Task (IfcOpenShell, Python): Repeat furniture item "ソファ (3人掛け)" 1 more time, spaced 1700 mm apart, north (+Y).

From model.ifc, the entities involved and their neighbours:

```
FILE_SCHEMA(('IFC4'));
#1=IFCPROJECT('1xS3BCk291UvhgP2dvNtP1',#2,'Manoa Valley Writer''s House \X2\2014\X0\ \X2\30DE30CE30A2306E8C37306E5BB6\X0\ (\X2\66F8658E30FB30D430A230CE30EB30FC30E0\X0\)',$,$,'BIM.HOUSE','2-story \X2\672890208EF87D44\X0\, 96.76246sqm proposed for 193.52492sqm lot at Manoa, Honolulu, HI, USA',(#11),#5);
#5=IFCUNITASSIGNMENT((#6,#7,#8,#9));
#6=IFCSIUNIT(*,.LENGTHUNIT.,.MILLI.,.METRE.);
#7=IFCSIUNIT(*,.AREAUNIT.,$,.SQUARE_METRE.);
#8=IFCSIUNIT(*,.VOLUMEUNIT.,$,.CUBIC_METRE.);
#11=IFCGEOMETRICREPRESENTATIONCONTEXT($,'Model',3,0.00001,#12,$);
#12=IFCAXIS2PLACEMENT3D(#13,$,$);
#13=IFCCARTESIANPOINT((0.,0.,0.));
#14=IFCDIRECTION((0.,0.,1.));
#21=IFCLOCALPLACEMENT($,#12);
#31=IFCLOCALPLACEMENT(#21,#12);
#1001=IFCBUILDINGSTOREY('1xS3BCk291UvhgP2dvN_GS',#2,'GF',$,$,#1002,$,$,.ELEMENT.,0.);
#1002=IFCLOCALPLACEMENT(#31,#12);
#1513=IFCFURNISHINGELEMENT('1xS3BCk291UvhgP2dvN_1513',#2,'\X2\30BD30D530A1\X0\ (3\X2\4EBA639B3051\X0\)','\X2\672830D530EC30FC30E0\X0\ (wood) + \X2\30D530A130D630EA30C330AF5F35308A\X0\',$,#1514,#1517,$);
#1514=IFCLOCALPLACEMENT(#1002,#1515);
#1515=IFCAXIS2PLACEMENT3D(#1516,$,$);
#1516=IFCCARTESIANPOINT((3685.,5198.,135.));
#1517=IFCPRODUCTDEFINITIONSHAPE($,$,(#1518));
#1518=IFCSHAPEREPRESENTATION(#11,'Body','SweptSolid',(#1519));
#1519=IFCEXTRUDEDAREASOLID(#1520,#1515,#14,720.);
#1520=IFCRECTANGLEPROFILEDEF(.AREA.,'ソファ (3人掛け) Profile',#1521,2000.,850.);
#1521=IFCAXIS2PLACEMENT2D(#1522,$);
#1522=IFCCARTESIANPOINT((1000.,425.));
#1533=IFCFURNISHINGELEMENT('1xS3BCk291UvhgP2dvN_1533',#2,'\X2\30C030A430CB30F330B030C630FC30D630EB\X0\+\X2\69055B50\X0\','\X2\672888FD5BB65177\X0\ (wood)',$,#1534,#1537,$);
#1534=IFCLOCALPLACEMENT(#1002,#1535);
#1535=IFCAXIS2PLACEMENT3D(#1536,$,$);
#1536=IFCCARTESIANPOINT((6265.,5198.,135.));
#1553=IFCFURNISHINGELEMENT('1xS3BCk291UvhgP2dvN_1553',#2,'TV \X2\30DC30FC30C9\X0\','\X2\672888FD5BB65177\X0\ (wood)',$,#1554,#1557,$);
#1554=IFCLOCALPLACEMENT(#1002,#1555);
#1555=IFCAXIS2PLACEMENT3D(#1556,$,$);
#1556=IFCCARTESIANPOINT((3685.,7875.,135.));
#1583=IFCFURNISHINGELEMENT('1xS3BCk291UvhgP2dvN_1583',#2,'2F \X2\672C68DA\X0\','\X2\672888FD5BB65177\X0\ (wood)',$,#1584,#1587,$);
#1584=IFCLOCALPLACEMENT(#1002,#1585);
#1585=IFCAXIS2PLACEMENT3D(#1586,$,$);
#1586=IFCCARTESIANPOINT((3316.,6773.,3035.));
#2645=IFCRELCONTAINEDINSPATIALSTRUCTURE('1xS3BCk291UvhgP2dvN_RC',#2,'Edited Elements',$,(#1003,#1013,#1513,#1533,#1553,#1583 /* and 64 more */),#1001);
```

```python
import numpy as np
import ifcopenshell
import ifcopenshell.api.geometry
import ifcopenshell.api.root
import ifcopenshell.util.element
import ifcopenshell.util.placement

model = ifcopenshell.open("model.ifc")


def reuse_history(source, copy):
    """copy_class also copies each property set's owner history, people and application; keep the originals."""
    for rel in copy.IsDefinedBy:
        if rel.is_a("IfcRelDefinesByProperties") and (history := rel.RelatingPropertyDefinition.OwnerHistory):
            rel.RelatingPropertyDefinition.OwnerHistory = source.OwnerHistory
            ifcopenshell.util.element.remove_deep2(model, history)


source = model.by_guid("1xS3BCk291UvhgP2dvN_1513")
base = ifcopenshell.util.placement.get_local_placement(source.ObjectPlacement)
step = np.array([0.0, 1.0, 0.0]) * 1700.0

for i in range(1, 2):
    copy = ifcopenshell.api.root.copy_class(model, product=source)
    copy.Representation = ifcopenshell.util.element.copy_deep(
        model, source.Representation, exclude=["IfcGeometricRepresentationContext", "IfcRepresentationMap"]
    )
    reuse_history(source, copy)
    matrix = base.copy()
    matrix[:3, 3] += i * step
    print("added at", matrix[:3, 3].round(3) + 0.0)
    ifcopenshell.api.geometry.edit_object_placement(model, product=copy, matrix=matrix, is_si=False)

model.write("model-out.ifc")
```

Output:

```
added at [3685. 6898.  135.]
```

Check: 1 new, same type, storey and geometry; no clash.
